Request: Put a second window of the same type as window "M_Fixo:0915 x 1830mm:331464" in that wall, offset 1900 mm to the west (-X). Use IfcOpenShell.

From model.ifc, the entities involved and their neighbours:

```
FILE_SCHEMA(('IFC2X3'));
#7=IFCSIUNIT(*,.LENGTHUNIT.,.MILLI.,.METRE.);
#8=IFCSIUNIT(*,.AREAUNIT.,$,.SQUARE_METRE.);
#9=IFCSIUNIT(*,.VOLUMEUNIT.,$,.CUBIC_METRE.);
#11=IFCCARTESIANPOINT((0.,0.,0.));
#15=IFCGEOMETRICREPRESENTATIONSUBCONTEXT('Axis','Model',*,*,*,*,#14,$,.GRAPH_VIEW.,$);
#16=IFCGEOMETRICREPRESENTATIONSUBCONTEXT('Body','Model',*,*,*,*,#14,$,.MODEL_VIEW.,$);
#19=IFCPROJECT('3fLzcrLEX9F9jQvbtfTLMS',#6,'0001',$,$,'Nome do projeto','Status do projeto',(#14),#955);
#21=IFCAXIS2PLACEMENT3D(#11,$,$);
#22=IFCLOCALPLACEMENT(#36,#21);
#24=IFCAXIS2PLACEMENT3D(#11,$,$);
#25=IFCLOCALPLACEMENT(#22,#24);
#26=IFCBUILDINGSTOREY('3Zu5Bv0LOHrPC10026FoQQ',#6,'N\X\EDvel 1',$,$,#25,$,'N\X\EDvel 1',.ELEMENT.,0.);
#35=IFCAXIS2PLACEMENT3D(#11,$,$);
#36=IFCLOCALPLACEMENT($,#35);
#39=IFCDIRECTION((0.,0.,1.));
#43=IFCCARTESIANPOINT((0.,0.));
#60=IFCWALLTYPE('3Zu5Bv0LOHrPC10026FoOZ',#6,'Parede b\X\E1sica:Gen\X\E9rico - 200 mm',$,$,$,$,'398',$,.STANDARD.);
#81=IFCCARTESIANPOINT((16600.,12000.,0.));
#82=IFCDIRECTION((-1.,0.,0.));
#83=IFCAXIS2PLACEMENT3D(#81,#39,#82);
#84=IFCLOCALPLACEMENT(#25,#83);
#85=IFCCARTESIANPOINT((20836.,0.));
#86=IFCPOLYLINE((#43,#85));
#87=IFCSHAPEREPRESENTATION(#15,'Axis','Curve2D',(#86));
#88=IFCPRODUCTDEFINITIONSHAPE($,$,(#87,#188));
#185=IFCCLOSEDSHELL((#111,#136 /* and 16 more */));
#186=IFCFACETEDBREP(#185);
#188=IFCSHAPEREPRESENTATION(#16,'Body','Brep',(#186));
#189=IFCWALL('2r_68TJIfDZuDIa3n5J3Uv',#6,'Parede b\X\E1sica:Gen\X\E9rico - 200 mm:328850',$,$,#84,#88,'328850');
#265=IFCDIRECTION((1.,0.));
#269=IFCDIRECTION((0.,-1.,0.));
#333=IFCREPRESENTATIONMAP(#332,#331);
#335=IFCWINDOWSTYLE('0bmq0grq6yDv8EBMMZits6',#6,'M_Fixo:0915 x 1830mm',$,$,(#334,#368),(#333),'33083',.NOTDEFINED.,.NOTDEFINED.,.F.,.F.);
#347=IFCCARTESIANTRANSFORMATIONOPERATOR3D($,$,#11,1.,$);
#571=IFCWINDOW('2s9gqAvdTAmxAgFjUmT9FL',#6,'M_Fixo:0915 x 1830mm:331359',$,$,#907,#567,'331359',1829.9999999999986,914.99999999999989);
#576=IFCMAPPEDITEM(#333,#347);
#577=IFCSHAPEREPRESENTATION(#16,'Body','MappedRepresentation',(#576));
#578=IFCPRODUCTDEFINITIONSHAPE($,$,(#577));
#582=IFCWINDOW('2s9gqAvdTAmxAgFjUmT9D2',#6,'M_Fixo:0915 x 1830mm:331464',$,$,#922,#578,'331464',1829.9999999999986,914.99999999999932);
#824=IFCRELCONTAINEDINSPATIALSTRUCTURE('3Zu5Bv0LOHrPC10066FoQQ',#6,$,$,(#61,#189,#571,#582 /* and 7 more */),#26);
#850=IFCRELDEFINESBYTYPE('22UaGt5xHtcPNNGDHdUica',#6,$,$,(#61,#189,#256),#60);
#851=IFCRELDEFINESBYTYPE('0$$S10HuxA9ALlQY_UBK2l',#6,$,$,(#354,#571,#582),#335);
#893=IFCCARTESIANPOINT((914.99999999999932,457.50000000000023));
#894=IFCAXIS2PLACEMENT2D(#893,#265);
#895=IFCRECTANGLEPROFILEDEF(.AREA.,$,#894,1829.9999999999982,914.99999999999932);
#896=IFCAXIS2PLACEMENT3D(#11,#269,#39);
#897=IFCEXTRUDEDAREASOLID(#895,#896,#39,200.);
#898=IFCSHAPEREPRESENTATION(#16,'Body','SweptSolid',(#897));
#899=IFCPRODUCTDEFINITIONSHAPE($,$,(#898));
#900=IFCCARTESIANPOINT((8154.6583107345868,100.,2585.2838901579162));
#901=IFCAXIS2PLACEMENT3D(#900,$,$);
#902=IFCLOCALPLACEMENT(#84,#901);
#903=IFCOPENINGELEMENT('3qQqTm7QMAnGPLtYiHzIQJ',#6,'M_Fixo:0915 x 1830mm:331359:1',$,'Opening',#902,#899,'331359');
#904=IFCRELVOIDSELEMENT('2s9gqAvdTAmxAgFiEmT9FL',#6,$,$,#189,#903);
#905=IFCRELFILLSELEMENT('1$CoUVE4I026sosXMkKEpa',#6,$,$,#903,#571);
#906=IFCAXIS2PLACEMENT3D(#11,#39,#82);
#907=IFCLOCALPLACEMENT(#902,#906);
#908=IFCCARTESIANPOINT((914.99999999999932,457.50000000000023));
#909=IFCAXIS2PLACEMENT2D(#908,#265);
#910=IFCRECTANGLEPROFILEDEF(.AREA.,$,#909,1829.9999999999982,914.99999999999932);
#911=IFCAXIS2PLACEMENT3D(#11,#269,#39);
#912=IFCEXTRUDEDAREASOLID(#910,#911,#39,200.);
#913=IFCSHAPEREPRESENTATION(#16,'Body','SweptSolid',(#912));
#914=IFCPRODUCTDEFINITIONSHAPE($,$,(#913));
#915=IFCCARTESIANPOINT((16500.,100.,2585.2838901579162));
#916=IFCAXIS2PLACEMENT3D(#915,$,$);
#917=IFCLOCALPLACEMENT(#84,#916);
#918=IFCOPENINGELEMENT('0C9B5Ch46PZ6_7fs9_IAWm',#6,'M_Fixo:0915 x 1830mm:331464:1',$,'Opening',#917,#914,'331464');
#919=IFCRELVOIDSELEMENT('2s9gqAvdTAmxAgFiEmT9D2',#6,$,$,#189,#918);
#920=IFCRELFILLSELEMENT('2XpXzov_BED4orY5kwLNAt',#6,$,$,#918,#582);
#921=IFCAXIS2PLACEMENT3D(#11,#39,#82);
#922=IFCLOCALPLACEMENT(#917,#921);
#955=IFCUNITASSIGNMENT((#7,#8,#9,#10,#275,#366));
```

```python
import ifcopenshell
import ifcopenshell.api.feature
import ifcopenshell.api.geometry
import ifcopenshell.api.root
import ifcopenshell.geom
import ifcopenshell.util.element
import ifcopenshell.util.placement
import ifcopenshell.util.shape

model = ifcopenshell.open("model.ifc")
settings = ifcopenshell.geom.settings()


def volume(element):
    """Net volume in cubic metres, openings subtracted."""
    shape = ifcopenshell.geom.create_shape(settings, element)
    return ifcopenshell.util.shape.get_volume(shape.geometry)


def reuse_history(source, copy):
    """copy_class also copies each property set's owner history, people and application; keep the originals."""
    for rel in copy.IsDefinedBy:
        if rel.is_a("IfcRelDefinesByProperties") and (history := rel.RelatingPropertyDefinition.OwnerHistory):
            rel.RelatingPropertyDefinition.OwnerHistory = source.OwnerHistory
            ifcopenshell.util.element.remove_deep2(model, history)


window = model.by_guid("2s9gqAvdTAmxAgFjUmT9D2")
opening = window.FillsVoids[0].RelatingOpeningElement
wall = opening.VoidsElements[0].RelatingBuildingElement
before = volume(wall)
shift = ifcopenshell.util.placement.get_local_placement(wall.ObjectPlacement)[:3, 0] * 1900.0

# copy_class copies the void relationship, type, container and properties, but no geometry.
new_opening = ifcopenshell.api.root.copy_class(model, product=opening)
new_opening.Representation = ifcopenshell.util.element.copy_deep(
    model, opening.Representation, exclude=["IfcGeometricRepresentationContext", "IfcRepresentationMap"]
)
new_opening.Name = "M_Fixo:0915 x 1830mm"
new_opening.Tag = None
new_window = ifcopenshell.api.root.copy_class(model, product=window)
new_window.Representation = ifcopenshell.util.element.copy_deep(
    model, window.Representation, exclude=["IfcGeometricRepresentationContext", "IfcRepresentationMap"]
)
new_window.Name = "M_Fixo:0915 x 1830mm"
new_window.Tag = None
reuse_history(window, new_window)
fills = ifcopenshell.api.feature.add_filling(model, opening=new_opening, element=new_window)
fills.OwnerHistory = new_window.OwnerHistory  # required in IFC2X3

for old, new in ((opening, new_opening), (window, new_window)):
    matrix = ifcopenshell.util.placement.get_local_placement(old.ObjectPlacement)
    matrix[:3, 3] += shift
    ifcopenshell.api.geometry.edit_object_placement(model, product=new, matrix=matrix, is_si=False)

after = volume(wall)

print(f"wall volume {before:.3f} -> {after:.3f} m3")

model.write("model_updated.ifc")
```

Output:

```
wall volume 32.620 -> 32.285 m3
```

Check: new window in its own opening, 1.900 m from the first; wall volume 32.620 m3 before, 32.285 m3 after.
